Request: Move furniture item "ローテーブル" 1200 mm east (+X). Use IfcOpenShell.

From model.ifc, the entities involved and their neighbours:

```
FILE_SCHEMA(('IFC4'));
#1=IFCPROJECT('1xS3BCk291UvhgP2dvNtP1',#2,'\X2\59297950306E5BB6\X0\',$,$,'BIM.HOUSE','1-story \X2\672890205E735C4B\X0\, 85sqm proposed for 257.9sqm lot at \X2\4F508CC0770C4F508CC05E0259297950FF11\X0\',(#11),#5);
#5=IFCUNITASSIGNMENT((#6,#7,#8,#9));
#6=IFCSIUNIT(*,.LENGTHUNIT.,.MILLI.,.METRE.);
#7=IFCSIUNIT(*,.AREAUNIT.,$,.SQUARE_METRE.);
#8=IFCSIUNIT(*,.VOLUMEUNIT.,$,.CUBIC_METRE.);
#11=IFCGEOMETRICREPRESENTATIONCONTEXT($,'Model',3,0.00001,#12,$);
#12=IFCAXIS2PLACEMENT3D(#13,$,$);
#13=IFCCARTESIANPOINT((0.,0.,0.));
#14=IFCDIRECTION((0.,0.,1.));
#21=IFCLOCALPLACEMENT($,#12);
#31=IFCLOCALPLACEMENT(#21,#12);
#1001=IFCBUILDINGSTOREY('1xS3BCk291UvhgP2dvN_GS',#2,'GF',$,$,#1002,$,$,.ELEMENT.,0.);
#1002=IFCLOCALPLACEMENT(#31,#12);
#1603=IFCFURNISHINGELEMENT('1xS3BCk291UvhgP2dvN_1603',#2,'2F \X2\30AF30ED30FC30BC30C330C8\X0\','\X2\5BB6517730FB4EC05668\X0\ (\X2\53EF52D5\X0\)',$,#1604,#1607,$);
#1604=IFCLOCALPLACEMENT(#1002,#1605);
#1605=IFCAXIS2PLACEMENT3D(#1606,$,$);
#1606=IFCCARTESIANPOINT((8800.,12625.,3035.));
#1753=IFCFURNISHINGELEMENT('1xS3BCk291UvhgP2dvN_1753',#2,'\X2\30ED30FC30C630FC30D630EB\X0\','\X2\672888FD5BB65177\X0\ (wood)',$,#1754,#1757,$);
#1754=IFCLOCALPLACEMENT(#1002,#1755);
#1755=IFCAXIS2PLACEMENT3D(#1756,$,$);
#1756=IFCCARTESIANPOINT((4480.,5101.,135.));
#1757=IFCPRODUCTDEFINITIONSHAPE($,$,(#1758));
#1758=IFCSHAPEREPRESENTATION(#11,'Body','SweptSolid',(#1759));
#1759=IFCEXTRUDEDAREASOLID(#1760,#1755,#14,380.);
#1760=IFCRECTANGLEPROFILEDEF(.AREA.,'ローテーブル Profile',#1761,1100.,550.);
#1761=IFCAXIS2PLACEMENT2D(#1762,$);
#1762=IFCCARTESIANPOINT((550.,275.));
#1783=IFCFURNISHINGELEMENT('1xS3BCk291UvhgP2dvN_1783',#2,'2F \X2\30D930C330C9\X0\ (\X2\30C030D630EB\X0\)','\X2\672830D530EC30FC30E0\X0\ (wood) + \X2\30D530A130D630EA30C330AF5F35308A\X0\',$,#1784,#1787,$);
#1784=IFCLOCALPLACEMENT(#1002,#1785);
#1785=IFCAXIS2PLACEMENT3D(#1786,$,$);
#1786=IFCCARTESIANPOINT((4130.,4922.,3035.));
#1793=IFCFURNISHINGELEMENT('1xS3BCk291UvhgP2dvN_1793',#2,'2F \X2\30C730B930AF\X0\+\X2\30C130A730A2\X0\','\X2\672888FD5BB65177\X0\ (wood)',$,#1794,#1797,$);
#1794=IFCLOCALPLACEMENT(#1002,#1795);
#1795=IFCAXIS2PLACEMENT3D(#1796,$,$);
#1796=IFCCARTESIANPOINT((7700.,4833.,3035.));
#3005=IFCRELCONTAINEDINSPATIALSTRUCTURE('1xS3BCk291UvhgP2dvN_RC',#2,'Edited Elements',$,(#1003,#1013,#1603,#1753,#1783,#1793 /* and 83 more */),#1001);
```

```python
import ifcopenshell
import ifcopenshell.api.geometry
import ifcopenshell.util.placement

model = ifcopenshell.open("model.ifc")

item = model.by_guid("1xS3BCk291UvhgP2dvN_1753")
matrix = ifcopenshell.util.placement.get_local_placement(item.ObjectPlacement)
matrix[0, 3] += 1200.0
ifcopenshell.api.geometry.edit_object_placement(model, product=item, matrix=matrix, is_si=False)

print(ifcopenshell.util.placement.get_local_placement(item.ObjectPlacement).round(3) + 0.0)

model.write("model_edited.ifc")
```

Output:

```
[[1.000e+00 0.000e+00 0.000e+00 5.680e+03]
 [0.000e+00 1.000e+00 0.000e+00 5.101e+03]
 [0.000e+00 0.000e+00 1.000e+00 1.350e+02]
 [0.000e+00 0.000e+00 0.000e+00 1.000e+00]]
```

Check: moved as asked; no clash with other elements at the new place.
